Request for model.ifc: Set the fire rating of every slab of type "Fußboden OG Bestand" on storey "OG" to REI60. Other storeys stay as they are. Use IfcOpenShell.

First a look at what the model holds.

```python
import ifcopenshell
import ifcopenshell.util.element

model = ifcopenshell.open("model.ifc")
print(model.schema)
storey = next(s for s in model.by_type("IfcBuildingStorey") if s.Name == "OG")
slabs = [e for e in ifcopenshell.util.element.get_decomposition(storey) if e.is_a("IfcSlab")]
seen = {}
for e in slabs:
    element_type = ifcopenshell.util.element.get_type(e)
    key = (element_type.Name if element_type != e and element_type else None, ifcopenshell.util.element.get_pset(e, "Pset_SlabCommon", "FireRating"))
    seen[key] = seen.get(key, 0) + 1
for (name, value), count in sorted(seen.items(), key=str):
    print(count, "x", name, "|", value)
```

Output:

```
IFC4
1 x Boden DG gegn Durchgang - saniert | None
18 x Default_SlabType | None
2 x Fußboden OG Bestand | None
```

```python
import ifcopenshell
import ifcopenshell.api.pset
import ifcopenshell.util.element

model = ifcopenshell.open("model.ifc")

storey = next(s for s in model.by_type("IfcBuildingStorey") if s.Name == "OG")
slabs = [e for e in ifcopenshell.util.element.get_decomposition(storey) if e.is_a("IfcSlab")]

count = 0
for e in slabs:
    element_type = ifcopenshell.util.element.get_type(e)
    if element_type in (None, e) or element_type.Name != "Fußboden OG Bestand":
        continue
    # add_pset returns the element's existing set when there is one.
    pset = ifcopenshell.api.pset.add_pset(model, product=e, name="Pset_SlabCommon")
    ifcopenshell.api.pset.edit_pset(model, pset=pset, properties={"FireRating": "REI60"})
    count += 1

print(count, "slabs updated")

model.write("model_edited.ifc")
```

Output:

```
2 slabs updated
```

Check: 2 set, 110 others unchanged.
